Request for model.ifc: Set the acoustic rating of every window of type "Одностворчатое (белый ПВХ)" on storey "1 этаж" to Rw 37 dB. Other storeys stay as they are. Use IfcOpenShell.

First a look at what the model holds.

```python
import ifcopenshell
import ifcopenshell.util.element

model = ifcopenshell.open("model.ifc")
print(model.schema)
storey = next(s for s in model.by_type("IfcBuildingStorey") if s.Name == "1 этаж")
windows = [e for e in ifcopenshell.util.element.get_decomposition(storey) if e.is_a("IfcWindow")]
seen = {}
for e in windows:
    element_type = ifcopenshell.util.element.get_type(e)
    key = (element_type.Name if element_type != e and element_type else None, ifcopenshell.util.element.get_pset(e, "Pset_WindowCommon", "AcousticRating"))
    seen[key] = seen.get(key, 0) + 1
for (name, value), count in sorted(seen.items(), key=str):
    print(count, "x", name, "|", value)
```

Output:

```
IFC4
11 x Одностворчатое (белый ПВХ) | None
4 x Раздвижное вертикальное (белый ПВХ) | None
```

```python
import ifcopenshell
import ifcopenshell.api.pset
import ifcopenshell.util.element

model = ifcopenshell.open("model.ifc")

storey = next(s for s in model.by_type("IfcBuildingStorey") if s.Name == "1 этаж")
windows = [e for e in ifcopenshell.util.element.get_decomposition(storey) if e.is_a("IfcWindow")]

count = 0
for e in windows:
    element_type = ifcopenshell.util.element.get_type(e)
    if element_type in (None, e) or element_type.Name != "Одностворчатое (белый ПВХ)":
        continue
    # add_pset returns the element's existing set when there is one.
    pset = ifcopenshell.api.pset.add_pset(model, product=e, name="Pset_WindowCommon")
    ifcopenshell.api.pset.edit_pset(model, pset=pset, properties={"AcousticRating": "Rw 37 dB"})
    count += 1

print(count, "windows updated")

model.write("model_v2.ifc")
```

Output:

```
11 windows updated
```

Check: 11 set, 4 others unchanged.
